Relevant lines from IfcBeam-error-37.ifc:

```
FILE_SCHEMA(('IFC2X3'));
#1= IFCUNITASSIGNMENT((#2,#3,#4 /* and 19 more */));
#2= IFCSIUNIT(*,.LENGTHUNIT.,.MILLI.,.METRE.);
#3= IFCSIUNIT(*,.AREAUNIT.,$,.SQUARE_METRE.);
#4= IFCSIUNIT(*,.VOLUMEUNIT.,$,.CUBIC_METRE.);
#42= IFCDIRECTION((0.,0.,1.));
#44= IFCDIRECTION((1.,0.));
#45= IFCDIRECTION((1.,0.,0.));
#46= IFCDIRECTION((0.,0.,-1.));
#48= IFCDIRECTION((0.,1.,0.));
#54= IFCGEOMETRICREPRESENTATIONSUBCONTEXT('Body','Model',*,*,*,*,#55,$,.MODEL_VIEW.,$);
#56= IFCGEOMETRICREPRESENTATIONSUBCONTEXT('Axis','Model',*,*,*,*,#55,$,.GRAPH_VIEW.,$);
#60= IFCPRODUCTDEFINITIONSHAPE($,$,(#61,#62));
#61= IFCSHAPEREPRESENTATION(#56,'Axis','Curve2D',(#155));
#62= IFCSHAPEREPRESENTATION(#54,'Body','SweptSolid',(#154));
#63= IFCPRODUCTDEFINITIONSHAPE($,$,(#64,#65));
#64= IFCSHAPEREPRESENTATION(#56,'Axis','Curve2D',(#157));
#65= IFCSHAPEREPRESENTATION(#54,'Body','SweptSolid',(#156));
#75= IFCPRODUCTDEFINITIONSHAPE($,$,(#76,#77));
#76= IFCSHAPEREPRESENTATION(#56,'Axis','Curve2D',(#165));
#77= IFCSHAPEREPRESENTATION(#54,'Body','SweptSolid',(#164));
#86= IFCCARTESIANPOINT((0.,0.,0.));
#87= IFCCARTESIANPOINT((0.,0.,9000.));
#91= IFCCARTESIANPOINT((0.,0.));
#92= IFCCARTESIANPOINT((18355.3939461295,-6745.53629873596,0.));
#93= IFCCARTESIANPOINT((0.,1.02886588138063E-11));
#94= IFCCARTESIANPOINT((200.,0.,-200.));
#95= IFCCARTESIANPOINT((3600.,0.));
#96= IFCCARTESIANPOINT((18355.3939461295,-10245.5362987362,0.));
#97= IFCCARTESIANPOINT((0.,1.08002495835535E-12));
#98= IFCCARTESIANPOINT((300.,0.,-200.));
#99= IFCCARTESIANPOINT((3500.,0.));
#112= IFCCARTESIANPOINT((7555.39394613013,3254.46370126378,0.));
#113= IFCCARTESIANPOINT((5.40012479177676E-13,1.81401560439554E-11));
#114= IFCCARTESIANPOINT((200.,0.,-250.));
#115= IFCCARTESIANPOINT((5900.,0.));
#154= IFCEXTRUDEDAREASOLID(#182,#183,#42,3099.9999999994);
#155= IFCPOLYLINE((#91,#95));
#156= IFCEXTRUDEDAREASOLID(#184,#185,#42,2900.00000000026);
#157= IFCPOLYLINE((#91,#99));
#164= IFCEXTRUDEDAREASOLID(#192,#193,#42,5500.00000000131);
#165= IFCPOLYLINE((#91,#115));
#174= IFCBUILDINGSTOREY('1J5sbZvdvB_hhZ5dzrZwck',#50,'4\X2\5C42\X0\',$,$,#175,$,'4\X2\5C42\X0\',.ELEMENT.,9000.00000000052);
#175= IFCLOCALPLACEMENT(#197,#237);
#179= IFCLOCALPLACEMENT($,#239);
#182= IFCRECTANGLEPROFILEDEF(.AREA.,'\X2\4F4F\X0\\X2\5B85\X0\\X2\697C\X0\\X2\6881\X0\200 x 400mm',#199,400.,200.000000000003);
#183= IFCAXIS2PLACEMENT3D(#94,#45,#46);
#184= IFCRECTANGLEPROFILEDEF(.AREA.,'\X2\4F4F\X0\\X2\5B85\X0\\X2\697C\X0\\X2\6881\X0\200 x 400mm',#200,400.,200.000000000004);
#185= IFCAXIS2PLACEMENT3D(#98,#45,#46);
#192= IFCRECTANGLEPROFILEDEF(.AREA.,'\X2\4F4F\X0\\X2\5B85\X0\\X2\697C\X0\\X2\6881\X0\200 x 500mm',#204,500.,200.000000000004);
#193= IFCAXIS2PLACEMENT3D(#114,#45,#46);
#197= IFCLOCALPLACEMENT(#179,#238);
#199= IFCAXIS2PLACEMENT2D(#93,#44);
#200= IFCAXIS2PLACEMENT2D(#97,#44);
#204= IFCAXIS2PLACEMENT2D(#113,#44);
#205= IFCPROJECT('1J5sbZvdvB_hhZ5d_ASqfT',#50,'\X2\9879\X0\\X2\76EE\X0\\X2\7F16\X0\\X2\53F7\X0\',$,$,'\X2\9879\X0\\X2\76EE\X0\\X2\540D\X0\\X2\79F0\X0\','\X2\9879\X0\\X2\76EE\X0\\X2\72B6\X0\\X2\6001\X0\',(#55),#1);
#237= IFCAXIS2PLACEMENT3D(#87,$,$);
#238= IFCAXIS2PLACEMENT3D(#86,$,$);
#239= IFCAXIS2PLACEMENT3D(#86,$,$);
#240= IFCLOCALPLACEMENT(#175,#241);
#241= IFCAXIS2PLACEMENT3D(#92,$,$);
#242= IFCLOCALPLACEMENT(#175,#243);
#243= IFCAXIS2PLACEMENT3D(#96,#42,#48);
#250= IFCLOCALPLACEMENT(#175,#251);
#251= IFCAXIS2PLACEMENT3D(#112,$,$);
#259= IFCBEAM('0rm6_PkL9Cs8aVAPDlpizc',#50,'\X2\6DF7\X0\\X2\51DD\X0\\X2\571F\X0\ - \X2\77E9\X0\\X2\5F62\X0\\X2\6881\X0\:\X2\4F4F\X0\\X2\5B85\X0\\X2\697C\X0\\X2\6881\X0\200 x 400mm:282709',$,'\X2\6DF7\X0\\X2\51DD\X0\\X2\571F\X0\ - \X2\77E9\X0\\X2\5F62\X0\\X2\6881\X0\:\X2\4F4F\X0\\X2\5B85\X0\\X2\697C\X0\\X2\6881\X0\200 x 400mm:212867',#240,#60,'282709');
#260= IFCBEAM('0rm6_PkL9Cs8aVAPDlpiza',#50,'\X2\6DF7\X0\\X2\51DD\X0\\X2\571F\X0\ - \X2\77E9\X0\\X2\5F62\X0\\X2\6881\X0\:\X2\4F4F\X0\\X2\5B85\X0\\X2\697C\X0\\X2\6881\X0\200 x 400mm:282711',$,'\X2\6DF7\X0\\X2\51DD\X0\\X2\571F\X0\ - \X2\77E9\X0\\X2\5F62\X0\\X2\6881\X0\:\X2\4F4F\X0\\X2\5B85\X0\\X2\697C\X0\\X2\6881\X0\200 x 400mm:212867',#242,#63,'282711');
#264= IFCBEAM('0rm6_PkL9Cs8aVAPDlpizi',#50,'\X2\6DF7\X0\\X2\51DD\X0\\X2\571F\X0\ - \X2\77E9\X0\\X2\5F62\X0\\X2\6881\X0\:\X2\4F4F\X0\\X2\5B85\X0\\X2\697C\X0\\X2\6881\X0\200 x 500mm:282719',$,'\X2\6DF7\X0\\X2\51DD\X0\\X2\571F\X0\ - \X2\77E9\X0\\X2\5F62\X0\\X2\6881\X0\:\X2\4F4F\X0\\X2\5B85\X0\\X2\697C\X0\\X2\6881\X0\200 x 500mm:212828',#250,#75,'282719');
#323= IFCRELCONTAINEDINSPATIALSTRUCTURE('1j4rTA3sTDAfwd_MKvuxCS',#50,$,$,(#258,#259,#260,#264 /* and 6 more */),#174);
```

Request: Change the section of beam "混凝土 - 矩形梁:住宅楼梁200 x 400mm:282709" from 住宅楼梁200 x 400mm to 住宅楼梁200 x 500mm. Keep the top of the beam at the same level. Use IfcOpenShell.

```python
import ifcopenshell
import ifcopenshell.util.element
import ifcopenshell.util.representation

model = ifcopenshell.open("IfcBeam-error-37.ifc")

member = model.by_guid("0rm6_PkL9Cs8aVAPDlpizc")
source = next(p for p in model.by_type("IfcRectangleProfileDef") if p.ProfileName == "住宅楼梁200 x 500mm")

body = ifcopenshell.util.representation.get_representation(member, "Model", "Body")
solid = body.Items[0]
old_profile = solid.SweptArea

# Copy the section's sizes but keep this member's own profile position.
profile = ifcopenshell.util.element.copy(model, source)
# Profiles are centred, so shift by half the change in depth to hold the top.
shift = (old_profile.XDim - profile.XDim) / 2
x, y = old_profile.Position.Location.Coordinates
up = (-1.0, 0.0)  # upwards, in the solid's own plane
location = model.createIfcCartesianPoint((x + up[0] * shift, y + up[1] * shift))
profile.Position = model.createIfcAxis2Placement2D(location, old_profile.Position.RefDirection)
solid.SweptArea = profile
if not model.get_total_inverses(old_profile):
    ifcopenshell.util.element.remove_deep2(model, old_profile)
member.Name = member.Name.replace("住宅楼梁200 x 400mm", "住宅楼梁200 x 500mm")
member.ObjectType = member.ObjectType.replace("住宅楼梁200 x 400mm", "住宅楼梁200 x 500mm")

print(solid.SweptArea)

model.write("IfcBeam-error-37-out.ifc")
```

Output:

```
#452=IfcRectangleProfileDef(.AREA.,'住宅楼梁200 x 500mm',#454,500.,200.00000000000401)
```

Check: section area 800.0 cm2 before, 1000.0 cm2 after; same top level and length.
